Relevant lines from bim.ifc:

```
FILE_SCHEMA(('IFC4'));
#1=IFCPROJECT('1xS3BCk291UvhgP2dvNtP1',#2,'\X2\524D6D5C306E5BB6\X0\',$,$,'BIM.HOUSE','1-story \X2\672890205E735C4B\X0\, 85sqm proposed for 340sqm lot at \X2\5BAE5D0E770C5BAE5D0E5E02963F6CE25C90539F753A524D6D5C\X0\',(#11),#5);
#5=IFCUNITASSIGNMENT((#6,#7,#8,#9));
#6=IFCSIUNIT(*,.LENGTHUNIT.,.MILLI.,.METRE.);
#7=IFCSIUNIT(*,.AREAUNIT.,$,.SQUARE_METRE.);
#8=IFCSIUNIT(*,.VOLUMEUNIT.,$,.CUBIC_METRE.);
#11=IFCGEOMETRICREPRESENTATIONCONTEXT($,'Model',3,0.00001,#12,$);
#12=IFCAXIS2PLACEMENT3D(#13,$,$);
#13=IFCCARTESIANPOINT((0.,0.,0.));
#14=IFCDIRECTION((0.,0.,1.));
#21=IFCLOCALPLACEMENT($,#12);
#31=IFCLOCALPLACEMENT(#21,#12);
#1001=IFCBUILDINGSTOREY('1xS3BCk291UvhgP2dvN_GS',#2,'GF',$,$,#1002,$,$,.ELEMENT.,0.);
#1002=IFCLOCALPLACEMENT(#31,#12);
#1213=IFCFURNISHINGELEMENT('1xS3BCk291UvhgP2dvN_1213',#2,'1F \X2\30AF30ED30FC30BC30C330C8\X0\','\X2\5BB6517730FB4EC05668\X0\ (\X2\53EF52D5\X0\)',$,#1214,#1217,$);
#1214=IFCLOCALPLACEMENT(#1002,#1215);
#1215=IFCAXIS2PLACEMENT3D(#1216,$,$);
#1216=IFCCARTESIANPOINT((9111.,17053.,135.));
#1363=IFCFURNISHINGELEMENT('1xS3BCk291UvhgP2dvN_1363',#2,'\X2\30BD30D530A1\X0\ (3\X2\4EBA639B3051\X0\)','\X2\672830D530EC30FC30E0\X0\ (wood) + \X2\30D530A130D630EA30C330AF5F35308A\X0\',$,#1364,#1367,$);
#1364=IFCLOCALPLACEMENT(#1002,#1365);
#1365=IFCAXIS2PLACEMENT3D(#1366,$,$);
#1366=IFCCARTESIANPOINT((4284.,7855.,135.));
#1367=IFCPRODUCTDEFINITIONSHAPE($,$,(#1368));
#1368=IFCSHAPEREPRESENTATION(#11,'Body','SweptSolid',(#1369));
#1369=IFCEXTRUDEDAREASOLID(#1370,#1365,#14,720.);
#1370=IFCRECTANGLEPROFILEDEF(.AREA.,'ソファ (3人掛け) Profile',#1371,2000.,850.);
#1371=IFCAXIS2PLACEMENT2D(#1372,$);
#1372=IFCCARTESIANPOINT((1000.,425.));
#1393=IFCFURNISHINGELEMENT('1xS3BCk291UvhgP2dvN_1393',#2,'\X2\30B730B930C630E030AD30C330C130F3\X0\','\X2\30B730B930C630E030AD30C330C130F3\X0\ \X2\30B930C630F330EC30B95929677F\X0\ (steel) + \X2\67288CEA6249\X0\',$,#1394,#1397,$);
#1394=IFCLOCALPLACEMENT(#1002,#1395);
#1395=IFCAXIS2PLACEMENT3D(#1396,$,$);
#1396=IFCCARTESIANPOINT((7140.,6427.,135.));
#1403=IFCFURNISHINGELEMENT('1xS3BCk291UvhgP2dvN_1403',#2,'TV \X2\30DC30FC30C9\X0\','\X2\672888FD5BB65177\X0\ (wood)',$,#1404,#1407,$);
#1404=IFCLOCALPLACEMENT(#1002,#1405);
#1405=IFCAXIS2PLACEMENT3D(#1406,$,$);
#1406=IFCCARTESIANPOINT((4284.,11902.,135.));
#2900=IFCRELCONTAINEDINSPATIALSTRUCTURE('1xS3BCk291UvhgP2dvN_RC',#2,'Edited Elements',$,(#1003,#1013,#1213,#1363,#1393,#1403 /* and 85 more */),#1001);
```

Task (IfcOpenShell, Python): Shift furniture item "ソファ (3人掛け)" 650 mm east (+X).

```python
import ifcopenshell
import ifcopenshell.api.geometry
import ifcopenshell.util.placement

model = ifcopenshell.open("bim.ifc")

item = model.by_guid("1xS3BCk291UvhgP2dvN_1363")
matrix = ifcopenshell.util.placement.get_local_placement(item.ObjectPlacement)
matrix[0, 3] += 650.0
ifcopenshell.api.geometry.edit_object_placement(model, product=item, matrix=matrix, is_si=False)

print(ifcopenshell.util.placement.get_local_placement(item.ObjectPlacement).round(3) + 0.0)

model.write("bim_updated.ifc")
```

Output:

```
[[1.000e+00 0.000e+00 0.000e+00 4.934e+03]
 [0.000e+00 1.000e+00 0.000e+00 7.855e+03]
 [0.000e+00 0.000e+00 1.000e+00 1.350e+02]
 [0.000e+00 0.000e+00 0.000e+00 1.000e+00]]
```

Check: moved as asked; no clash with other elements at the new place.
